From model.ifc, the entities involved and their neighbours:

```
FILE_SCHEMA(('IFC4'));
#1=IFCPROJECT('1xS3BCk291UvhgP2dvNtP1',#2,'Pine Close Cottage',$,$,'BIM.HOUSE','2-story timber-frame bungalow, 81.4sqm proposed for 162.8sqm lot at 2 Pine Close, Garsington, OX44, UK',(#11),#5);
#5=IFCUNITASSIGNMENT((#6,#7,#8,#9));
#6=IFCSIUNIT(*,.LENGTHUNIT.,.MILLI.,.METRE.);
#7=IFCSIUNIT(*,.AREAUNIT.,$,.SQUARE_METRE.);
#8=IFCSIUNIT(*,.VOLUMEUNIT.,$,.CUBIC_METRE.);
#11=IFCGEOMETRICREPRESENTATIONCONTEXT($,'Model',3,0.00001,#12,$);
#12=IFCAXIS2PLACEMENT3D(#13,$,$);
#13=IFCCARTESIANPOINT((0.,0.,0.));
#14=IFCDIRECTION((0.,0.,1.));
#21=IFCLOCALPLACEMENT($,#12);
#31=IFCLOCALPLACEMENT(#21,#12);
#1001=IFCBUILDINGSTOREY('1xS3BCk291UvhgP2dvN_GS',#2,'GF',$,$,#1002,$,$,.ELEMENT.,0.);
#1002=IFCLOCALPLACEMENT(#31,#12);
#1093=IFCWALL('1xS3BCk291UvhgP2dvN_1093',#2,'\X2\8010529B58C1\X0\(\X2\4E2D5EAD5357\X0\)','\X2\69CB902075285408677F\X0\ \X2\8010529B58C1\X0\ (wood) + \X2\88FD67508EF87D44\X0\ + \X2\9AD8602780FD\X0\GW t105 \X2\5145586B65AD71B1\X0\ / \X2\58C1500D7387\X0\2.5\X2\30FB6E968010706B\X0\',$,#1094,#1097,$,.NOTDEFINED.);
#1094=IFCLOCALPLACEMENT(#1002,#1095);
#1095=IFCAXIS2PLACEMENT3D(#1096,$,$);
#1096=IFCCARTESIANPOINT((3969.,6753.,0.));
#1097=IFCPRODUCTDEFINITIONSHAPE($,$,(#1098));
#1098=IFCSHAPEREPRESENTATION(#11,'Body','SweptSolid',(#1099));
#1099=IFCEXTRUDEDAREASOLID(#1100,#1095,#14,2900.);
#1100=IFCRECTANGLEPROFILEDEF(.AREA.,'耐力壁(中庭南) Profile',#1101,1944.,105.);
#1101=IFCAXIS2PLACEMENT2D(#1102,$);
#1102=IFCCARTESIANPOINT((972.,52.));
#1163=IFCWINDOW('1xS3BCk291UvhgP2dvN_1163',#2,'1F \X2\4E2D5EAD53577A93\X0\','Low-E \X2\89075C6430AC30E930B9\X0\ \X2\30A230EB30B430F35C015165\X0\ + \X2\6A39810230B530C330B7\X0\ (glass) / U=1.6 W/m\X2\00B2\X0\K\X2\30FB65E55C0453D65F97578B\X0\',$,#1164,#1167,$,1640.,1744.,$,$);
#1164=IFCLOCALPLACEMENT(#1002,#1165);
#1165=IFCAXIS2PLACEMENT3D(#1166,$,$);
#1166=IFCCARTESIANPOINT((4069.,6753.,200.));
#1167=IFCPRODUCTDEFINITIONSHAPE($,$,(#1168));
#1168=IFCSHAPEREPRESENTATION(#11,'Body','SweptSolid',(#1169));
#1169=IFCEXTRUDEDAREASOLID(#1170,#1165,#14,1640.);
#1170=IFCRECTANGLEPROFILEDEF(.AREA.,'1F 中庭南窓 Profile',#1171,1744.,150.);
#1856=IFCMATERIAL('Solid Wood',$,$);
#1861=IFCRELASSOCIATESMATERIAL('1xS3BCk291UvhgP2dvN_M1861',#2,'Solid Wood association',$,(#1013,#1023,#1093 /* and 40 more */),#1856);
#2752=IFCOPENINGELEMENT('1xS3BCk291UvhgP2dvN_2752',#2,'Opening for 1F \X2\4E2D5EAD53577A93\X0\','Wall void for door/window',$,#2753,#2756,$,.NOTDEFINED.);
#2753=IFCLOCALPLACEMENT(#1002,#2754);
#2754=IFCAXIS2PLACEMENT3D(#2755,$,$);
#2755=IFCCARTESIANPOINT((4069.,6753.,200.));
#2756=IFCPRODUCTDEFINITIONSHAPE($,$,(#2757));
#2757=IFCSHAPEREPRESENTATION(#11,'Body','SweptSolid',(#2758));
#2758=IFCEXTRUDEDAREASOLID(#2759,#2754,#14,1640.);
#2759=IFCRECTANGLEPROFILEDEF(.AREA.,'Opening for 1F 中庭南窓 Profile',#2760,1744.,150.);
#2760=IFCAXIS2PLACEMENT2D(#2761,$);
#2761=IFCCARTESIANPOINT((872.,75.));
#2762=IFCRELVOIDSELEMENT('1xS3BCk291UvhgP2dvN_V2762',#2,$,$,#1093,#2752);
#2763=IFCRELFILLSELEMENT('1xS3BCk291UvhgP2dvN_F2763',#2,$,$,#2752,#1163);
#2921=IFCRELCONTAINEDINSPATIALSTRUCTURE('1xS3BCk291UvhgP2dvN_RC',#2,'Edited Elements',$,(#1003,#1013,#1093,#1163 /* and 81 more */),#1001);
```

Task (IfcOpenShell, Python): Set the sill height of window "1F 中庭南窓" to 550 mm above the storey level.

```python
import numpy as np
import ifcopenshell
import ifcopenshell.api.geometry
import ifcopenshell.geom
import ifcopenshell.util.element
import ifcopenshell.util.placement
import ifcopenshell.util.shape
import ifcopenshell.util.unit

model = ifcopenshell.open("model.ifc")
unit_scale = ifcopenshell.util.unit.calculate_unit_scale(model)

window = model.by_guid("1xS3BCk291UvhgP2dvN_1163")
opening = window.FillsVoids[0].RelatingOpeningElement
storey = ifcopenshell.util.element.get_container(window, ifc_class="IfcBuildingStorey")
level = ifcopenshell.util.placement.get_local_placement(storey.ObjectPlacement)[2, 3]

# The opening's origin need not be at the sill, so measure its lowest point.
shape = ifcopenshell.geom.create_shape(ifcopenshell.geom.settings(), opening)
bottom = ifcopenshell.util.shape.get_shape_bottom_elevation(shape, shape.geometry) / unit_scale
dz = level + 550.0 - bottom

shift = np.array([0.0, 0.0, dz])
# The window is not placed relative to its opening, so move both.
for product in (opening, window):
    matrix = ifcopenshell.util.placement.get_local_placement(product.ObjectPlacement)
    matrix[:3, 3] += shift
    ifcopenshell.api.geometry.edit_object_placement(model, product=product, matrix=matrix, is_si=False)

print(f"moved by {dz * unit_scale:+.3f} m")

model.write("model_v2.ifc")
```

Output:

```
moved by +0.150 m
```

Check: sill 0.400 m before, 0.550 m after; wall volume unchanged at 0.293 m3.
